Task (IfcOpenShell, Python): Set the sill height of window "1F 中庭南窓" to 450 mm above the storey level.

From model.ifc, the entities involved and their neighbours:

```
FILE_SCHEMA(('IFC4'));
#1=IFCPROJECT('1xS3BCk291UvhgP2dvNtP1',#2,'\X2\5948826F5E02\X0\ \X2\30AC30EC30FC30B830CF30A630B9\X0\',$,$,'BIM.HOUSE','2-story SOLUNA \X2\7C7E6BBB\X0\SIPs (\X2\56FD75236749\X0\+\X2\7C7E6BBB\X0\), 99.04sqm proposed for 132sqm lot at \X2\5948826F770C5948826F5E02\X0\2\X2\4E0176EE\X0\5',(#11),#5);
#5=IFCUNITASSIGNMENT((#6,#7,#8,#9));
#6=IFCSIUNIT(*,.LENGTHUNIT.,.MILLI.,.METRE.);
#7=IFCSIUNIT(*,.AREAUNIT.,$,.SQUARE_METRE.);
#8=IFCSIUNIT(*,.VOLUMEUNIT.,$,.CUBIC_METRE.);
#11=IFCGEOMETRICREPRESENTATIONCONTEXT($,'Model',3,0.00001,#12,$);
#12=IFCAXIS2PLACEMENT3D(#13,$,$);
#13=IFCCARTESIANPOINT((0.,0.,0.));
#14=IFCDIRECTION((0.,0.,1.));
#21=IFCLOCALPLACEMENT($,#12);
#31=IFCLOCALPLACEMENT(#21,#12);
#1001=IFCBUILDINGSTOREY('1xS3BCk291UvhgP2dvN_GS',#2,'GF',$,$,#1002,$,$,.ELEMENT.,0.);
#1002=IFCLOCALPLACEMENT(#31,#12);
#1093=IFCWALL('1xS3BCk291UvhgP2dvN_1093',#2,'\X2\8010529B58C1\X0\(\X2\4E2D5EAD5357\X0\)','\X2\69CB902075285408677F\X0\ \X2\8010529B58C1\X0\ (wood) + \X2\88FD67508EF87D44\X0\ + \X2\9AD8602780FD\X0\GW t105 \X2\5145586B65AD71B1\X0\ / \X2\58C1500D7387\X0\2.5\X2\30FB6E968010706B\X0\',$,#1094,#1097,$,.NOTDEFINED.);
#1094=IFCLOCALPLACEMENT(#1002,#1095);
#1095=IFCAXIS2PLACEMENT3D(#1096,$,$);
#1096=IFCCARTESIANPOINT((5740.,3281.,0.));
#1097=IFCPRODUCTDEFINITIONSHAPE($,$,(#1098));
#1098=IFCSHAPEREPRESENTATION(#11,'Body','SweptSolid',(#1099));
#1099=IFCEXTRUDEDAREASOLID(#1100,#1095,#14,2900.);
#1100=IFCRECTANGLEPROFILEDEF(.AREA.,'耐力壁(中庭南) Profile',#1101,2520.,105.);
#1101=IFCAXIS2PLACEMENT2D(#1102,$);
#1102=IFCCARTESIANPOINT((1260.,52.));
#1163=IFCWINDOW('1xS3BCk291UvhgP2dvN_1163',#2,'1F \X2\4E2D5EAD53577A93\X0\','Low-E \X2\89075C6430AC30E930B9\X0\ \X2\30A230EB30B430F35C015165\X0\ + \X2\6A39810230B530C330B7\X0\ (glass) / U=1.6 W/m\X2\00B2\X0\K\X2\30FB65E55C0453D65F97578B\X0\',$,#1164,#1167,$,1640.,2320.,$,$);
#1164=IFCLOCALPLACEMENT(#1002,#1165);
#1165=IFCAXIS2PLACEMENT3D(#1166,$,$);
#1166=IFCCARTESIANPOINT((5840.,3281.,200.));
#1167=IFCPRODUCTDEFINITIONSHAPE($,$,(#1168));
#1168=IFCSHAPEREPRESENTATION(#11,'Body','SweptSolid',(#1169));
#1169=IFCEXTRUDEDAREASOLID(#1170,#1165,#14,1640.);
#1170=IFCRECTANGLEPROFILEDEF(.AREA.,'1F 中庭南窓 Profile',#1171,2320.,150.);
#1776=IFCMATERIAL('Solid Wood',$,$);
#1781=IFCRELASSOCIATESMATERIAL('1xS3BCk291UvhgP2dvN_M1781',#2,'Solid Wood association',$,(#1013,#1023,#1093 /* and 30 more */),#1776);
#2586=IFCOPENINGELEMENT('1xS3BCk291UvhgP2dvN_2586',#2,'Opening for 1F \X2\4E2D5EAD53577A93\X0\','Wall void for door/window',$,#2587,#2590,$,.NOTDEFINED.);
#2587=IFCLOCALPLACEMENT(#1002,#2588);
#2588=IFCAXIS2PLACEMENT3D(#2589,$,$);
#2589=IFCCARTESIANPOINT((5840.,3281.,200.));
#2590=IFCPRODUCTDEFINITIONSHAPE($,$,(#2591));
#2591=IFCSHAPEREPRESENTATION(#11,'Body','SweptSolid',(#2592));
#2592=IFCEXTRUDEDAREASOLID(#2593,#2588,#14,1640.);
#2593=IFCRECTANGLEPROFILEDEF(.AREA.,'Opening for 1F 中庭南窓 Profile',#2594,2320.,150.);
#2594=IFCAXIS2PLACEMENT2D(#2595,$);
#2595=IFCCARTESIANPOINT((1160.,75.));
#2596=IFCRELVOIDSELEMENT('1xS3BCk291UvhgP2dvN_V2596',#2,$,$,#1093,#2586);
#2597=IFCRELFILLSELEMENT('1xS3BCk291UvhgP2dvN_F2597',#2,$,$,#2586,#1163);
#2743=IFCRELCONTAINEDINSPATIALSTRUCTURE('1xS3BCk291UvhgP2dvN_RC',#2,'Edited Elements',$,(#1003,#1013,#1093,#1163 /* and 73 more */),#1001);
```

```python
import numpy as np
import ifcopenshell
import ifcopenshell.api.geometry
import ifcopenshell.geom
import ifcopenshell.util.element
import ifcopenshell.util.placement
import ifcopenshell.util.shape
import ifcopenshell.util.unit

model = ifcopenshell.open("model.ifc")
unit_scale = ifcopenshell.util.unit.calculate_unit_scale(model)

window = model.by_guid("1xS3BCk291UvhgP2dvN_1163")
opening = window.FillsVoids[0].RelatingOpeningElement
storey = ifcopenshell.util.element.get_container(window, ifc_class="IfcBuildingStorey")
level = ifcopenshell.util.placement.get_local_placement(storey.ObjectPlacement)[2, 3]

# The opening's origin need not be at the sill, so measure its lowest point.
shape = ifcopenshell.geom.create_shape(ifcopenshell.geom.settings(), opening)
bottom = ifcopenshell.util.shape.get_shape_bottom_elevation(shape, shape.geometry) / unit_scale
dz = level + 0.45 / unit_scale - bottom

shift = np.array([0.0, 0.0, dz])
# The window is not placed relative to its opening, so move both.
for product in (opening, window):
    matrix = ifcopenshell.util.placement.get_local_placement(product.ObjectPlacement)
    matrix[:3, 3] += shift
    ifcopenshell.api.geometry.edit_object_placement(model, product=product, matrix=matrix, is_si=False)

print(f"moved by {dz * unit_scale:+.3f} m")

model.write("model_v2.ifc")
```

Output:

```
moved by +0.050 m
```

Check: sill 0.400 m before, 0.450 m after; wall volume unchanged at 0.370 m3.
